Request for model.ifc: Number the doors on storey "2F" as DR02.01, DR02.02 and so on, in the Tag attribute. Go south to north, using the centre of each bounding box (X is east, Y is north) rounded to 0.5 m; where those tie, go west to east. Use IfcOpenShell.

First a look at what the model holds.

```python
import ifcopenshell
import ifcopenshell.util.element
import ifcopenshell.util.placement

model = ifcopenshell.open("model.ifc")
print(model.schema)
storey = next(s for s in model.by_type("IfcBuildingStorey") if s.Name == "2F")
doors = [e for e in ifcopenshell.util.element.get_decomposition(storey) if e.is_a("IfcDoor")]
for e in sorted(doors, key=lambda e: e.id()):
    origin = ifcopenshell.util.placement.get_local_placement(e.ObjectPlacement)[:3, 3]
    print(e.id(), e.Tag, e.Name, origin.round(2) + 0.0, sep=" | ")
```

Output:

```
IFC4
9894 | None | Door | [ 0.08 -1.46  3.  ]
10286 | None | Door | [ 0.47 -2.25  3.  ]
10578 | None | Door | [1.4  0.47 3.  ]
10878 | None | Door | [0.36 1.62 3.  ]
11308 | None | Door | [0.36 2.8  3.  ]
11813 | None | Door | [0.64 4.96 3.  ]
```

```python
import ifcopenshell
import ifcopenshell.geom
import ifcopenshell.util.element
import ifcopenshell.util.shape

model = ifcopenshell.open("model.ifc")
settings = ifcopenshell.geom.settings()
settings.set("use-world-coords", True)


def centre(element):
    shape = ifcopenshell.geom.create_shape(settings, element)
    return ifcopenshell.util.shape.get_bbox_centroid(shape.geometry)


storey = next(s for s in model.by_type("IfcBuildingStorey") if s.Name == "2F")
doors = [e for e in ifcopenshell.util.element.get_decomposition(storey) if e.is_a("IfcDoor")]

# Insertion points can sit at a corner or the storey origin, so sort by the geometry (in metres).
centres = {e: centre(e) for e in doors}
doors.sort(key=lambda e: (round(centres[e][1] / 0.5), centres[e][0]))

for i, e in enumerate(doors, start=1):
    number = f"DR02.{i:02d}"
    e.Tag = number
    print(e.id(), number)

model.write("model-out.ifc")
```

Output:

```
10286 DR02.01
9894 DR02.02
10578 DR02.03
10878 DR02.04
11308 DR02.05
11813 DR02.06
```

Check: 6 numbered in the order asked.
